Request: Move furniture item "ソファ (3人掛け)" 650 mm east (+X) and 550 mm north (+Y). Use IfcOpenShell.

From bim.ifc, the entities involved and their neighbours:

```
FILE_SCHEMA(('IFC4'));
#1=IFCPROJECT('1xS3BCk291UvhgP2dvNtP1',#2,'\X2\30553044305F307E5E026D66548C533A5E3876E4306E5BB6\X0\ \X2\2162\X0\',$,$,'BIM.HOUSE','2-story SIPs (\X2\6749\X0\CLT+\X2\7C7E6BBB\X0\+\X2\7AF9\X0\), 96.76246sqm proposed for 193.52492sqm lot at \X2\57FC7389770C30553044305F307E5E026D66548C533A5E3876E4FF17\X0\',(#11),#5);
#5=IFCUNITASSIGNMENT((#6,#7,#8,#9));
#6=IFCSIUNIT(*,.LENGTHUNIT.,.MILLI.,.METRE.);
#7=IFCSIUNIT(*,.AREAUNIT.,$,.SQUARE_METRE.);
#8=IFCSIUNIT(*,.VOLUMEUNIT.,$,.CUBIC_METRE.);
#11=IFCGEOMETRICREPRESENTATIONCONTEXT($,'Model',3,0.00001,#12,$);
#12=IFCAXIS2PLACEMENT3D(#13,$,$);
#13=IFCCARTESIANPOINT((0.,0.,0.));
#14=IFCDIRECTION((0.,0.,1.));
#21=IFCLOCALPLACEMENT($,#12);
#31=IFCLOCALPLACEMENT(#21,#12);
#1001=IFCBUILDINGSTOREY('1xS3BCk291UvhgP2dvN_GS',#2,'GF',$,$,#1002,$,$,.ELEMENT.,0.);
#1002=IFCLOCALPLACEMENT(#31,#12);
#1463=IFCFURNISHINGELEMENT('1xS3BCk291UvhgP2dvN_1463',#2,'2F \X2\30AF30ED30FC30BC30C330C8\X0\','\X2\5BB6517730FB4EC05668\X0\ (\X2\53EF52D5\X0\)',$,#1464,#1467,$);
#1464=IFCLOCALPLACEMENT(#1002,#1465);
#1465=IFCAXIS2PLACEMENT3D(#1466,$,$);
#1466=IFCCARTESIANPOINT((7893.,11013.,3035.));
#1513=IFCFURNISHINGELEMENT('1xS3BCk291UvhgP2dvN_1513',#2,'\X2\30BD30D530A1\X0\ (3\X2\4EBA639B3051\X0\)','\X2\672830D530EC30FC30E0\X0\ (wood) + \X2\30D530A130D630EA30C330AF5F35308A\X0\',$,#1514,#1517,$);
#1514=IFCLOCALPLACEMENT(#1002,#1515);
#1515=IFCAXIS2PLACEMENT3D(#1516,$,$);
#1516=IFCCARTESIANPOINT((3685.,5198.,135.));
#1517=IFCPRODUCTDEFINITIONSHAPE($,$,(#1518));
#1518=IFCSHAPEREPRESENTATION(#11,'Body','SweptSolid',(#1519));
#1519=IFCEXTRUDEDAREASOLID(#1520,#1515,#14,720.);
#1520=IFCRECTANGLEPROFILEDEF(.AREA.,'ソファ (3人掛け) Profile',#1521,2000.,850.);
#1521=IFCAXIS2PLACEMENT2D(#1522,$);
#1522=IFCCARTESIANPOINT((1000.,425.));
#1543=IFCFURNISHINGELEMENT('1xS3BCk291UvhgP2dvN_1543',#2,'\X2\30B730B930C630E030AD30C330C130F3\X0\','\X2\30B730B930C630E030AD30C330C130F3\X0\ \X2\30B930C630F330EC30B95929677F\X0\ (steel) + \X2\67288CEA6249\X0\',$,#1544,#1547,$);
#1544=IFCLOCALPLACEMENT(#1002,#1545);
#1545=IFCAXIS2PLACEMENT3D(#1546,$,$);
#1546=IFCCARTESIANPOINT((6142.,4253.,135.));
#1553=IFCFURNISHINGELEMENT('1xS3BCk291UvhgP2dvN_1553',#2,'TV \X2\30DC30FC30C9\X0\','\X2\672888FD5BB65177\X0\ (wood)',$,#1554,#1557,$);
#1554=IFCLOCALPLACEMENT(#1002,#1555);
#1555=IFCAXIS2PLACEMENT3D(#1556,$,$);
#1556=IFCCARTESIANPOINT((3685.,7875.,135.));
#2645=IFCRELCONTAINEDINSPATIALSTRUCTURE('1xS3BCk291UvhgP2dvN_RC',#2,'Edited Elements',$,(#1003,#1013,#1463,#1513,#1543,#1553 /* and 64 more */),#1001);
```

```python
import ifcopenshell
import ifcopenshell.api.geometry
import ifcopenshell.util.placement
import ifcopenshell.util.unit

model = ifcopenshell.open("bim.ifc")
unit_scale = ifcopenshell.util.unit.calculate_unit_scale(model)

item = model.by_guid("1xS3BCk291UvhgP2dvN_1513")
matrix = ifcopenshell.util.placement.get_local_placement(item.ObjectPlacement)
matrix[0, 3] += 0.65 / unit_scale
matrix[1, 3] += 0.55 / unit_scale
ifcopenshell.api.geometry.edit_object_placement(model, product=item, matrix=matrix, is_si=False)

print(ifcopenshell.util.placement.get_local_placement(item.ObjectPlacement).round(3) + 0.0)

model.write("bim-out.ifc")
```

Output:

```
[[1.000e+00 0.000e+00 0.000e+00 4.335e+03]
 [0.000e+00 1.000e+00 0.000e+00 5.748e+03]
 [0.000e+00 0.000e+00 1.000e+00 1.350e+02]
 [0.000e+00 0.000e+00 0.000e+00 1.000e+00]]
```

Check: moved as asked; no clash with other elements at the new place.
